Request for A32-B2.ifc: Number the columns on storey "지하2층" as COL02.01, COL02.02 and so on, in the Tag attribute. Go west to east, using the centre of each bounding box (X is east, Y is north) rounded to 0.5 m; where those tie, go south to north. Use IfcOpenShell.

First a look at what the model holds.

```python
import ifcopenshell
import ifcopenshell.util.element
import ifcopenshell.util.placement

model = ifcopenshell.open("A32-B2.ifc")
print(model.schema)
storey = next(s for s in model.by_type("IfcBuildingStorey") if s.Name == "지하2층")
columns = [e for e in ifcopenshell.util.element.get_decomposition(storey) if e.is_a("IfcColumn")]
for e in sorted(columns, key=lambda e: e.id()):
    origin = ifcopenshell.util.placement.get_local_placement(e.ObjectPlacement)[:3, 3]
    print(e.id(), e.Tag, e.Name, origin.round(2) + 0.0, sep=" | ")
```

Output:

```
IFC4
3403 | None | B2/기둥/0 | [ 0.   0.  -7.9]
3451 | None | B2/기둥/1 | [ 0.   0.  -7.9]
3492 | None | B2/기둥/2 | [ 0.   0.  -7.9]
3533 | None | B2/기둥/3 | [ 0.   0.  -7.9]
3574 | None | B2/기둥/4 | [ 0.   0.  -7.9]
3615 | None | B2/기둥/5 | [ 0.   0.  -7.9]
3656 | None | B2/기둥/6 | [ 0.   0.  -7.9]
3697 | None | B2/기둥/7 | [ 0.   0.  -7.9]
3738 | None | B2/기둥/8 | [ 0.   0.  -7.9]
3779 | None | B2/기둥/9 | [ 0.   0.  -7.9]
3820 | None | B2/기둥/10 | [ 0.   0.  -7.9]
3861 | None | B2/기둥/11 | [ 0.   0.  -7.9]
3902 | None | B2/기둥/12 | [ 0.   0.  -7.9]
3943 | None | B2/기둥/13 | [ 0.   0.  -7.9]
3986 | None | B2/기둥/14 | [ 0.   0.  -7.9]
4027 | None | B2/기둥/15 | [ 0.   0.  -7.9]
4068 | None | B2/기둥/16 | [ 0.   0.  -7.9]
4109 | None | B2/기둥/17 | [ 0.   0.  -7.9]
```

```python
import ifcopenshell
import ifcopenshell.geom
import ifcopenshell.util.element
import ifcopenshell.util.shape

model = ifcopenshell.open("A32-B2.ifc")
settings = ifcopenshell.geom.settings()
settings.set("use-world-coords", True)


def centre(element):
    shape = ifcopenshell.geom.create_shape(settings, element)
    return ifcopenshell.util.shape.get_bbox_centroid(shape.geometry)


storey = next(s for s in model.by_type("IfcBuildingStorey") if s.Name == "지하2층")
columns = [e for e in ifcopenshell.util.element.get_decomposition(storey) if e.is_a("IfcColumn")]

# Insertion points can sit at a corner or the storey origin, so sort by the geometry (in metres).
centres = {e: centre(e) for e in columns}
columns.sort(key=lambda e: (round(centres[e][0] / 0.5), centres[e][1]))

for i, e in enumerate(columns, start=1):
    number = f"COL02.{i:02d}"
    e.Tag = number
    print(e.id(), number)

model.write("A32-B2_rev.ifc")
```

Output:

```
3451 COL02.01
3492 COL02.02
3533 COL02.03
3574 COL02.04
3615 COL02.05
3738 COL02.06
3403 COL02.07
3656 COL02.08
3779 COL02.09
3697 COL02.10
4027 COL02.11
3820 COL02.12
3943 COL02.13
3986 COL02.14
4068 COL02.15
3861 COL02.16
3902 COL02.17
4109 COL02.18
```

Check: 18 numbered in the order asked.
